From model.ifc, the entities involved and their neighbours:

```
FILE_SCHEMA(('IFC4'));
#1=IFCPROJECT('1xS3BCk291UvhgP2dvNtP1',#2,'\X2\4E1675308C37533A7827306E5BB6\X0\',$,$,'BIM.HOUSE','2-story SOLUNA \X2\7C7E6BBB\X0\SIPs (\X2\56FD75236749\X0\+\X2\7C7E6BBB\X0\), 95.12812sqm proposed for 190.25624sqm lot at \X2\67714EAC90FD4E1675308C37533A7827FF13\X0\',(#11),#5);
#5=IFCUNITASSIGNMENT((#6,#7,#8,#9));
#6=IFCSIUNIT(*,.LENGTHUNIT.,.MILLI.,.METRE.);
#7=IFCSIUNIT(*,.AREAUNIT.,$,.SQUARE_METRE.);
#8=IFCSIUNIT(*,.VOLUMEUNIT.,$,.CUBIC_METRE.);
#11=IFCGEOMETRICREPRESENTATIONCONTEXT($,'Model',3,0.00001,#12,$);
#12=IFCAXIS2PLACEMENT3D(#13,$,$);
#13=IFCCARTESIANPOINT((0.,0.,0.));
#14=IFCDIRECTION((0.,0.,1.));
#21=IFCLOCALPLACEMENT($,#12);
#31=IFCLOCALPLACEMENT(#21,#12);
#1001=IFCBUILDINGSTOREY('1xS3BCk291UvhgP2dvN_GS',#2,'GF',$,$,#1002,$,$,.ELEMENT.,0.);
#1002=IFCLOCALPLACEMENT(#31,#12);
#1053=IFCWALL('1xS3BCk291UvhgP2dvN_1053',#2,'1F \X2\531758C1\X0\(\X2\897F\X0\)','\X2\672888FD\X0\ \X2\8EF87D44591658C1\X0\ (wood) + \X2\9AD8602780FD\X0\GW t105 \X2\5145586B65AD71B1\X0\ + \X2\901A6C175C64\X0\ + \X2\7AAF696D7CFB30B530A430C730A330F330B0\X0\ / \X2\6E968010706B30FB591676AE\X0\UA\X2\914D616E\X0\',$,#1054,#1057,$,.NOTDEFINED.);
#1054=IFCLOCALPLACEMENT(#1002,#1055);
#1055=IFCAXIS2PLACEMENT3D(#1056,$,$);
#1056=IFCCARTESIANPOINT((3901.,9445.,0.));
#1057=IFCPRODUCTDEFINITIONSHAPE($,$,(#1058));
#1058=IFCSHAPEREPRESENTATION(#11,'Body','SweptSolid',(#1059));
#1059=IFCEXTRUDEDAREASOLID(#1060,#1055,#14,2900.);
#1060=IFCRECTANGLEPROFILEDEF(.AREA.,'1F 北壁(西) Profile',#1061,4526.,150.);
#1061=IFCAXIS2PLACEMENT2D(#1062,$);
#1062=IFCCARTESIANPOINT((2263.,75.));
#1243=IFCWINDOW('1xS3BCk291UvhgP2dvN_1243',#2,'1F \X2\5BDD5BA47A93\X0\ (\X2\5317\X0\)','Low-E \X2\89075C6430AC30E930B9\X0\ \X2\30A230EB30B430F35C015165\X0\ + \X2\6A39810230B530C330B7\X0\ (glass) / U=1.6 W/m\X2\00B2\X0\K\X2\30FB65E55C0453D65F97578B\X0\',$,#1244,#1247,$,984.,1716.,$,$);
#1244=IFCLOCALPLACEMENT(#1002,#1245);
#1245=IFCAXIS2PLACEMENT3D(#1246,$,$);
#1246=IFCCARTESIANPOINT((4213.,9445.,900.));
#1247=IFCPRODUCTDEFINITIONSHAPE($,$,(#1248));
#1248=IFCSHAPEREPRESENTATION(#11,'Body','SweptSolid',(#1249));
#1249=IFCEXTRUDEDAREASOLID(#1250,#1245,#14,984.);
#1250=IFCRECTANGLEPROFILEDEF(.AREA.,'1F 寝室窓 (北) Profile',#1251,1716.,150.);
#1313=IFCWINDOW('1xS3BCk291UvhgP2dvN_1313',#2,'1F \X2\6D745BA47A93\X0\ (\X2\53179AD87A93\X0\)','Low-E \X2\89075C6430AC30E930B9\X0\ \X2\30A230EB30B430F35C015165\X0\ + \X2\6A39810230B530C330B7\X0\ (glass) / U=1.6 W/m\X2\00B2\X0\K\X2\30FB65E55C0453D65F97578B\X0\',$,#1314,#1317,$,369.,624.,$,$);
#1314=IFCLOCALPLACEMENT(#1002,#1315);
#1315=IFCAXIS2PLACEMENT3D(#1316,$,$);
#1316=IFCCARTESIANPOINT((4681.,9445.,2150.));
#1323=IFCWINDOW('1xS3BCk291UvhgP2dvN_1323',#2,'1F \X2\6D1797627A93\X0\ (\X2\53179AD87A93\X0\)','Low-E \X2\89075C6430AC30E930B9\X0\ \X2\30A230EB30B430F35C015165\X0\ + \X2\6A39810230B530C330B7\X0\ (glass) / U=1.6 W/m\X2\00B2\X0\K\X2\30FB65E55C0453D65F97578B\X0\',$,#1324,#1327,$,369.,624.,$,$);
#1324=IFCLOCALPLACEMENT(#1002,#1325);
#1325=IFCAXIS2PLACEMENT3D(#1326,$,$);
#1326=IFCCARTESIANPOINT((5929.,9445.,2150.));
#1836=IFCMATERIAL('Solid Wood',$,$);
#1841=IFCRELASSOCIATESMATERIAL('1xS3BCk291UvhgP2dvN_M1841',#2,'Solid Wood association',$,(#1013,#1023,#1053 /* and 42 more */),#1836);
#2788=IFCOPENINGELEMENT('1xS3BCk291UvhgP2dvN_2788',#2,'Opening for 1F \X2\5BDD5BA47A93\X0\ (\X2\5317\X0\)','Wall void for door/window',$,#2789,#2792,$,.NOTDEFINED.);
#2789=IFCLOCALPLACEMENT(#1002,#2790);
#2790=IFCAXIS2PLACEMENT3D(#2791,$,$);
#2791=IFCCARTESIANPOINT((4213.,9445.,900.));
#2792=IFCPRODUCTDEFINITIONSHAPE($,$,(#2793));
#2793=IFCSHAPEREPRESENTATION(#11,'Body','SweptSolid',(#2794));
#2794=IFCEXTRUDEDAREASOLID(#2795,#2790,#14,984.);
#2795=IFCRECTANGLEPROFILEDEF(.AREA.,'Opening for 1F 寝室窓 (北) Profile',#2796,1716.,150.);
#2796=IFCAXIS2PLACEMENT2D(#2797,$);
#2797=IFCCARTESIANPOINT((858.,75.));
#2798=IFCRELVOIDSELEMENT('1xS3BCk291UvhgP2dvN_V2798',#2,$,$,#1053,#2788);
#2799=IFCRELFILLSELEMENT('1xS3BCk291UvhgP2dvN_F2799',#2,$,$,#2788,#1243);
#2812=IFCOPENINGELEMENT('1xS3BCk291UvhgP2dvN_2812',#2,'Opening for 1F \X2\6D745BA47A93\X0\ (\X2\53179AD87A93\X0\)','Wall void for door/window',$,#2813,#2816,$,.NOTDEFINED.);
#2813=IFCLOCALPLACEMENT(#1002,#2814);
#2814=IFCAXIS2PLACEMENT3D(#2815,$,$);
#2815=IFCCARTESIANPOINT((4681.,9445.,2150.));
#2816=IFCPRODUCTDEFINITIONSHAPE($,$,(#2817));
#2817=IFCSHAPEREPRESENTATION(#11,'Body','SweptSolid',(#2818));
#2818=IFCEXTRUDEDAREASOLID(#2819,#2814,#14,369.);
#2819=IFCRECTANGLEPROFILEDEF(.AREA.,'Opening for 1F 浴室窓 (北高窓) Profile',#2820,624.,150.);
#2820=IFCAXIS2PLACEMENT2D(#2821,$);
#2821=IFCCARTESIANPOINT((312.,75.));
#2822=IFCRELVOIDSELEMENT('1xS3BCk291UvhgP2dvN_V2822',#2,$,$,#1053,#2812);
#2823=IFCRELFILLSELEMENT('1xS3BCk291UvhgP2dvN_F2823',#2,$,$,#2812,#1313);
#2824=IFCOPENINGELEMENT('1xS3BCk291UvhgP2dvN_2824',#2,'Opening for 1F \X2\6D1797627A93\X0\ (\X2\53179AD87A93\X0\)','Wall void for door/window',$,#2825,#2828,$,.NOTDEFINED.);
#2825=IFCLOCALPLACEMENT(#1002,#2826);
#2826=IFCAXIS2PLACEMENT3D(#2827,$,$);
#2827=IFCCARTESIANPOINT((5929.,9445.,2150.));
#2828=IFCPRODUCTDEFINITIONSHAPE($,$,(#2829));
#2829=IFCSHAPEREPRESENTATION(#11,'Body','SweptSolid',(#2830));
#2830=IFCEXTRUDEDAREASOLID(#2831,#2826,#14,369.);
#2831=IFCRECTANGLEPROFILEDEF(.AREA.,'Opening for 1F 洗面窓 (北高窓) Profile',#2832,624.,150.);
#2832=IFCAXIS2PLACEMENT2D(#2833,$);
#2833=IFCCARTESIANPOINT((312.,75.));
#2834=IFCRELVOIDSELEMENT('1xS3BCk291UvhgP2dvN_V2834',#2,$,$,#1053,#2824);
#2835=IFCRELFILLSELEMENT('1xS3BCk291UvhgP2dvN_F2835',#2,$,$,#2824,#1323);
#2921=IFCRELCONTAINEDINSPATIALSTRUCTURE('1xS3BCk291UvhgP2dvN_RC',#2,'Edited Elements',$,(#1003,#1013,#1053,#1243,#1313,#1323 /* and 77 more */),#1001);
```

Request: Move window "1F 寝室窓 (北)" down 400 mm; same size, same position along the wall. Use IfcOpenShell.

```python
import numpy as np
import ifcopenshell
import ifcopenshell.api.geometry
import ifcopenshell.util.placement
import ifcopenshell.util.unit

model = ifcopenshell.open("model.ifc")
unit_scale = ifcopenshell.util.unit.calculate_unit_scale(model)

window = model.by_guid("1xS3BCk291UvhgP2dvN_1243")
opening = window.FillsVoids[0].RelatingOpeningElement
dz = -0.4 / unit_scale

shift = np.array([0.0, 0.0, dz])
# The window is not placed relative to its opening, so move both.
for product in (opening, window):
    matrix = ifcopenshell.util.placement.get_local_placement(product.ObjectPlacement)
    matrix[:3, 3] += shift
    ifcopenshell.api.geometry.edit_object_placement(model, product=product, matrix=matrix, is_si=False)

print(f"moved by {dz * unit_scale:+.3f} m")

model.write("model-out.ifc")
```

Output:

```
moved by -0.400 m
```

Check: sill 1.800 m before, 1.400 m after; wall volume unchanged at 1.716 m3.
